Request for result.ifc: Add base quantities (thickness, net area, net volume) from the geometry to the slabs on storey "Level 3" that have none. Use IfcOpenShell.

First a look at what the model holds.

```python
import ifcopenshell
import ifcopenshell.util.element
import ifcopenshell.util.unit

model = ifcopenshell.open("result.ifc")
print(model.schema)
for unit_type in ("LENGTHUNIT", "AREAUNIT", "VOLUMEUNIT"):
    print(unit_type, ifcopenshell.util.unit.calculate_unit_scale(model, unit_type))
storey = next(s for s in model.by_type("IfcBuildingStorey") if s.Name == "Level 3")
slabs = [e for e in ifcopenshell.util.element.get_decomposition(storey) if e.is_a("IfcSlab")]
for e in sorted(slabs, key=lambda e: e.id()):
    print(e.id(), e.is_a(), e.Name, list(ifcopenshell.util.element.get_psets(e, qtos_only=True)), sep=" | ")
```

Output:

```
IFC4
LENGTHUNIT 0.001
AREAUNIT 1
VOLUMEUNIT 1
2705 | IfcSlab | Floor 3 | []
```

```python
import ifcopenshell
import ifcopenshell.api.pset
import ifcopenshell.geom
import ifcopenshell.util.element
import ifcopenshell.util.shape
import ifcopenshell.util.unit

model = ifcopenshell.open("result.ifc")
unit_scale = ifcopenshell.util.unit.calculate_unit_scale(model)
area_scale = ifcopenshell.util.unit.calculate_unit_scale(model, "AREAUNIT")
volume_scale = ifcopenshell.util.unit.calculate_unit_scale(model, "VOLUMEUNIT")
settings = ifcopenshell.geom.settings()

storey = next(s for s in model.by_type("IfcBuildingStorey") if s.Name == "Level 3")
slabs = [e for e in ifcopenshell.util.element.get_decomposition(storey) if e.is_a("IfcSlab")]

for e in sorted(slabs, key=lambda e: e.id()):
    if ifcopenshell.util.element.get_psets(e, qtos_only=True, should_inherit=False):
        continue
    # Geometry comes back in metres, in the element's own axes.
    shape = ifcopenshell.geom.create_shape(settings, e)
    values = {
        "Width": ifcopenshell.util.shape.get_z(shape.geometry) / unit_scale,
        "NetArea": ifcopenshell.util.shape.get_footprint_area(shape.geometry) / area_scale,
        "NetVolume": ifcopenshell.util.shape.get_volume(shape.geometry) / volume_scale,
    }
    qto = ifcopenshell.api.pset.add_qto(model, product=e, name="Qto_SlabBaseQuantities")
    ifcopenshell.api.pset.edit_qto(model, qto=qto, properties=values)
    print(e.id(), {k: round(v, 3) for k, v in values.items()})

model.write("result_rev.ifc")
```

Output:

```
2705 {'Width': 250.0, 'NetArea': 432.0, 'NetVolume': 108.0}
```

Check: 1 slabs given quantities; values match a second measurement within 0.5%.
